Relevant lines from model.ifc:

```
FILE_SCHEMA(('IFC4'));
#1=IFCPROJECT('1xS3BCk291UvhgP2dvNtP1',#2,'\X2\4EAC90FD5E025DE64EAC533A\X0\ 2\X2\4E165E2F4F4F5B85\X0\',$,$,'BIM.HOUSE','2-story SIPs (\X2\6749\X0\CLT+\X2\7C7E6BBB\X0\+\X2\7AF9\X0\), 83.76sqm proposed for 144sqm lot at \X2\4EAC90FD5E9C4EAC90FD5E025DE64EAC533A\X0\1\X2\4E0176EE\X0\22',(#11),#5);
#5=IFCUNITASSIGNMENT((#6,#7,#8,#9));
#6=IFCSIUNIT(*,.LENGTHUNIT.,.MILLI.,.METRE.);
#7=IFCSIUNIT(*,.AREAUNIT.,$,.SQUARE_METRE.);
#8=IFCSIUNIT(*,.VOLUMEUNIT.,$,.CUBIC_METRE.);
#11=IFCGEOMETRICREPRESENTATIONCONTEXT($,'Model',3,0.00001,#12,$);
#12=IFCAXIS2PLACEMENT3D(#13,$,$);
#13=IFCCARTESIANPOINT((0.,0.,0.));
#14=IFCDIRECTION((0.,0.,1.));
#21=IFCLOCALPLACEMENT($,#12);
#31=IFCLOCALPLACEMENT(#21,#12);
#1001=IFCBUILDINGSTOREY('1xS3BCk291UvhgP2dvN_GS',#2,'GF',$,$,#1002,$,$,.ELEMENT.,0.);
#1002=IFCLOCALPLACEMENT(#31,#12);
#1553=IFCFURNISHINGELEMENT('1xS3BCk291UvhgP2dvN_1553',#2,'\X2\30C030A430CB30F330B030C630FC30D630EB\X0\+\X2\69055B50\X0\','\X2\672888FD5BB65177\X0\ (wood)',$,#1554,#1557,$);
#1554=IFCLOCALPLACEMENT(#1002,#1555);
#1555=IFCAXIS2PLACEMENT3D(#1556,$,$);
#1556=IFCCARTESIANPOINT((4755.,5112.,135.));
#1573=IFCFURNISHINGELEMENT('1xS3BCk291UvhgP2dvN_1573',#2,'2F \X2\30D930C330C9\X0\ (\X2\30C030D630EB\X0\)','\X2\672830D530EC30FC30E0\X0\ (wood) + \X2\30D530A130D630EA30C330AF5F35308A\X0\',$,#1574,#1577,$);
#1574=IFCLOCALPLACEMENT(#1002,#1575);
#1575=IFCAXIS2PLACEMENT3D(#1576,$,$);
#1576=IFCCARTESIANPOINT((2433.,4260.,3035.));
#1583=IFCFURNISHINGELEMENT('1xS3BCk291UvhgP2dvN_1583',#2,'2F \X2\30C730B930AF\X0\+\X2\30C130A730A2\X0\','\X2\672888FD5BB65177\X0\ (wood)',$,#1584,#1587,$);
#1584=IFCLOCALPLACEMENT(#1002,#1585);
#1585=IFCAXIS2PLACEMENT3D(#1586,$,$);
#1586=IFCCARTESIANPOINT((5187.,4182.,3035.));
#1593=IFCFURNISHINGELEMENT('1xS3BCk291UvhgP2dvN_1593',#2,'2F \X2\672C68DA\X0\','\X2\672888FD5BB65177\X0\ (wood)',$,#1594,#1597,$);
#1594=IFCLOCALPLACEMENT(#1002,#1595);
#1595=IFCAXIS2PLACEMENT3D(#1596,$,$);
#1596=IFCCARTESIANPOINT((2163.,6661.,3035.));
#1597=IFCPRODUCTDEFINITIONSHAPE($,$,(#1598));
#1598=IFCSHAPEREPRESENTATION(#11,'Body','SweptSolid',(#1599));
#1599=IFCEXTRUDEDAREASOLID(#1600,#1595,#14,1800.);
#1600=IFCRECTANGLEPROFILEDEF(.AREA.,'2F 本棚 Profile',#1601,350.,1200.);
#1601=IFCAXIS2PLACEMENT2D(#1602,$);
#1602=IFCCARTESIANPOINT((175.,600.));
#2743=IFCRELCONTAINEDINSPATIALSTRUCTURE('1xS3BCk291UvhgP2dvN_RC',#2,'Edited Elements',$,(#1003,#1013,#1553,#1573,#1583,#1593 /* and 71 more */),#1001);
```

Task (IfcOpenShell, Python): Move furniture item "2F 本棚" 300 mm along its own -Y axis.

```python
import ifcopenshell
import ifcopenshell.api.geometry
import ifcopenshell.util.placement

model = ifcopenshell.open("model.ifc")

item = model.by_guid("1xS3BCk291UvhgP2dvN_1593")
matrix = ifcopenshell.util.placement.get_local_placement(item.ObjectPlacement)
matrix[:3, 3] -= matrix[:3, 1] * 300.0
ifcopenshell.api.geometry.edit_object_placement(model, product=item, matrix=matrix, is_si=False)

print(ifcopenshell.util.placement.get_local_placement(item.ObjectPlacement).round(3) + 0.0)

model.write("model-out.ifc")
```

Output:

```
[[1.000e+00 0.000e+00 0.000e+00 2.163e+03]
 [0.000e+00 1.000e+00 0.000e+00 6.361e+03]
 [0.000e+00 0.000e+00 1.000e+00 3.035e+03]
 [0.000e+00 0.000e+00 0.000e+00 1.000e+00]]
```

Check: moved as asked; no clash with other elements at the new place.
